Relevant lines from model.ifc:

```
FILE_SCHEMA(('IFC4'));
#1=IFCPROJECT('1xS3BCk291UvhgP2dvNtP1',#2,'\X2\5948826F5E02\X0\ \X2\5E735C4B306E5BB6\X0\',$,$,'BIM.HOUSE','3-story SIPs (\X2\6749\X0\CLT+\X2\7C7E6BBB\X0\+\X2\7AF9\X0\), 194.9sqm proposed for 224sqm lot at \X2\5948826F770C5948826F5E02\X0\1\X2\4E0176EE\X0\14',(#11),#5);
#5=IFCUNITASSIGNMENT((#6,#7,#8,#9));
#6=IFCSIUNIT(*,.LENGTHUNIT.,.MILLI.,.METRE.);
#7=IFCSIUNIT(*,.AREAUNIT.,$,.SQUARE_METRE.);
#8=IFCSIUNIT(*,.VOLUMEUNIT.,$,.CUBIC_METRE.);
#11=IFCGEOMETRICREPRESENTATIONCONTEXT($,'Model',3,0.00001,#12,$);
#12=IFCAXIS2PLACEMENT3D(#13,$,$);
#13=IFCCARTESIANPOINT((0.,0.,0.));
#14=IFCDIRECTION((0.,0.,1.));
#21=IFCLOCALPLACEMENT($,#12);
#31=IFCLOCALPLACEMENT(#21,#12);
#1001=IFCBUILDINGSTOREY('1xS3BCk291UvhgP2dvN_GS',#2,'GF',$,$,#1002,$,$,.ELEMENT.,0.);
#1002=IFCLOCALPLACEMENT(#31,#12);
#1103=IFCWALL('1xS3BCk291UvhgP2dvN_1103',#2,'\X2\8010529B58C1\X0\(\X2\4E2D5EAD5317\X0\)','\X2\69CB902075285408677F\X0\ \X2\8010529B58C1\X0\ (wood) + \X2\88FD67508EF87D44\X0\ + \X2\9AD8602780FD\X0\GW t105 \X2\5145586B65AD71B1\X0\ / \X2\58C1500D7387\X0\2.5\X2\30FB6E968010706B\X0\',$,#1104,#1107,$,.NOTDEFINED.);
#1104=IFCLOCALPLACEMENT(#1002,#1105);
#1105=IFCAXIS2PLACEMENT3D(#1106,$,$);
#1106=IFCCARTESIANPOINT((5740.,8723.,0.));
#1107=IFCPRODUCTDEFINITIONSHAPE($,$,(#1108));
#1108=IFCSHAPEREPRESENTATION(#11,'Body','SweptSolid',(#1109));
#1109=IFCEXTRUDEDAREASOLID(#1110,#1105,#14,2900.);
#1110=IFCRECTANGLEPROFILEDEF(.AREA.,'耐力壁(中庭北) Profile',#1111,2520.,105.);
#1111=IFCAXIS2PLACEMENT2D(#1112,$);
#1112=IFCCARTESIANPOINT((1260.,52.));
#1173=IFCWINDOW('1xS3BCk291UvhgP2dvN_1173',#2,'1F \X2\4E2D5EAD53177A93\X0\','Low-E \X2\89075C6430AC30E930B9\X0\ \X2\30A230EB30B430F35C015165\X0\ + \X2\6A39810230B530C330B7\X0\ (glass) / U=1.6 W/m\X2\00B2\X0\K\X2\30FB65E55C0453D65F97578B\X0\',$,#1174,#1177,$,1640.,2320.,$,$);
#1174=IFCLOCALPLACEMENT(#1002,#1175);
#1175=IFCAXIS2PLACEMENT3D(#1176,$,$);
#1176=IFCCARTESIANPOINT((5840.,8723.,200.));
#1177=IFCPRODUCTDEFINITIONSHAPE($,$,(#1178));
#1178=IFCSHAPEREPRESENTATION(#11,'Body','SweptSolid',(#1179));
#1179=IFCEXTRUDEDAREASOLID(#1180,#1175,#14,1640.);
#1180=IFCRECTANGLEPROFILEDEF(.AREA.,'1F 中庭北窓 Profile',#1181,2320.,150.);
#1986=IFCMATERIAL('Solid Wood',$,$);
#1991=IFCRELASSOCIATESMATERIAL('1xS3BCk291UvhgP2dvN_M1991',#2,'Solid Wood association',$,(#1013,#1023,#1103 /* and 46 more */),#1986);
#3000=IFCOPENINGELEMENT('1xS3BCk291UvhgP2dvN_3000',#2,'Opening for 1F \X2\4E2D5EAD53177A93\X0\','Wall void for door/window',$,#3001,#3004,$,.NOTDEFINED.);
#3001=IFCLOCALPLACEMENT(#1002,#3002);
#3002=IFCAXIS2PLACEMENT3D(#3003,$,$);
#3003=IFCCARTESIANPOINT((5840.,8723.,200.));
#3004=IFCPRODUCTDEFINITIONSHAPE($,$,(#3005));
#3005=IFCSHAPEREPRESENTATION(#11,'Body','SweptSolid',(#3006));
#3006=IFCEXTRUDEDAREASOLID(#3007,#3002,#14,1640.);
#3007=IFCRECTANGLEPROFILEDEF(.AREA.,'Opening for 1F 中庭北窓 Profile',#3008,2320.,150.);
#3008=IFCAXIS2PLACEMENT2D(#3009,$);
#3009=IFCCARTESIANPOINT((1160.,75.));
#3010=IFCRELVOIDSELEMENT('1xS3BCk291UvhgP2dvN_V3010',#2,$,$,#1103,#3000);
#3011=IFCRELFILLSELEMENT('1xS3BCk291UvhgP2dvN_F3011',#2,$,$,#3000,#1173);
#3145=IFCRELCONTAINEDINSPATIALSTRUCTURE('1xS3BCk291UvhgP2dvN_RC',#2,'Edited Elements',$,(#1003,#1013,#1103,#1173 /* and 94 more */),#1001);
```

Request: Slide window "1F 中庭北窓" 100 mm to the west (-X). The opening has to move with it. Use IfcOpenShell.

```python
import ifcopenshell
import ifcopenshell.api.geometry
import ifcopenshell.util.placement
import ifcopenshell.util.unit

model = ifcopenshell.open("model.ifc")
unit_scale = ifcopenshell.util.unit.calculate_unit_scale(model)

window = model.by_guid("1xS3BCk291UvhgP2dvN_1173")
opening = window.FillsVoids[0].RelatingOpeningElement
wall = opening.VoidsElements[0].RelatingBuildingElement

wall_matrix = ifcopenshell.util.placement.get_local_placement(wall.ObjectPlacement)
shift = wall_matrix[:3, 0] * -0.1 / unit_scale
before = ifcopenshell.util.placement.get_local_placement(window.ObjectPlacement)[:3, 3].copy()

# The window is not placed relative to its opening, so move both.
for product in (opening, window):
    matrix = ifcopenshell.util.placement.get_local_placement(product.ObjectPlacement)
    matrix[:3, 3] += shift
    ifcopenshell.api.geometry.edit_object_placement(model, product=product, matrix=matrix, is_si=False)

after = ifcopenshell.util.placement.get_local_placement(window.ObjectPlacement)[:3, 3]
print("window moved by", (after - before).round(3) + 0.0)

model.write("model-out.ifc")
```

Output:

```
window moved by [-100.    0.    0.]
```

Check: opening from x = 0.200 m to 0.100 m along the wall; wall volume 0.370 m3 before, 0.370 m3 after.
